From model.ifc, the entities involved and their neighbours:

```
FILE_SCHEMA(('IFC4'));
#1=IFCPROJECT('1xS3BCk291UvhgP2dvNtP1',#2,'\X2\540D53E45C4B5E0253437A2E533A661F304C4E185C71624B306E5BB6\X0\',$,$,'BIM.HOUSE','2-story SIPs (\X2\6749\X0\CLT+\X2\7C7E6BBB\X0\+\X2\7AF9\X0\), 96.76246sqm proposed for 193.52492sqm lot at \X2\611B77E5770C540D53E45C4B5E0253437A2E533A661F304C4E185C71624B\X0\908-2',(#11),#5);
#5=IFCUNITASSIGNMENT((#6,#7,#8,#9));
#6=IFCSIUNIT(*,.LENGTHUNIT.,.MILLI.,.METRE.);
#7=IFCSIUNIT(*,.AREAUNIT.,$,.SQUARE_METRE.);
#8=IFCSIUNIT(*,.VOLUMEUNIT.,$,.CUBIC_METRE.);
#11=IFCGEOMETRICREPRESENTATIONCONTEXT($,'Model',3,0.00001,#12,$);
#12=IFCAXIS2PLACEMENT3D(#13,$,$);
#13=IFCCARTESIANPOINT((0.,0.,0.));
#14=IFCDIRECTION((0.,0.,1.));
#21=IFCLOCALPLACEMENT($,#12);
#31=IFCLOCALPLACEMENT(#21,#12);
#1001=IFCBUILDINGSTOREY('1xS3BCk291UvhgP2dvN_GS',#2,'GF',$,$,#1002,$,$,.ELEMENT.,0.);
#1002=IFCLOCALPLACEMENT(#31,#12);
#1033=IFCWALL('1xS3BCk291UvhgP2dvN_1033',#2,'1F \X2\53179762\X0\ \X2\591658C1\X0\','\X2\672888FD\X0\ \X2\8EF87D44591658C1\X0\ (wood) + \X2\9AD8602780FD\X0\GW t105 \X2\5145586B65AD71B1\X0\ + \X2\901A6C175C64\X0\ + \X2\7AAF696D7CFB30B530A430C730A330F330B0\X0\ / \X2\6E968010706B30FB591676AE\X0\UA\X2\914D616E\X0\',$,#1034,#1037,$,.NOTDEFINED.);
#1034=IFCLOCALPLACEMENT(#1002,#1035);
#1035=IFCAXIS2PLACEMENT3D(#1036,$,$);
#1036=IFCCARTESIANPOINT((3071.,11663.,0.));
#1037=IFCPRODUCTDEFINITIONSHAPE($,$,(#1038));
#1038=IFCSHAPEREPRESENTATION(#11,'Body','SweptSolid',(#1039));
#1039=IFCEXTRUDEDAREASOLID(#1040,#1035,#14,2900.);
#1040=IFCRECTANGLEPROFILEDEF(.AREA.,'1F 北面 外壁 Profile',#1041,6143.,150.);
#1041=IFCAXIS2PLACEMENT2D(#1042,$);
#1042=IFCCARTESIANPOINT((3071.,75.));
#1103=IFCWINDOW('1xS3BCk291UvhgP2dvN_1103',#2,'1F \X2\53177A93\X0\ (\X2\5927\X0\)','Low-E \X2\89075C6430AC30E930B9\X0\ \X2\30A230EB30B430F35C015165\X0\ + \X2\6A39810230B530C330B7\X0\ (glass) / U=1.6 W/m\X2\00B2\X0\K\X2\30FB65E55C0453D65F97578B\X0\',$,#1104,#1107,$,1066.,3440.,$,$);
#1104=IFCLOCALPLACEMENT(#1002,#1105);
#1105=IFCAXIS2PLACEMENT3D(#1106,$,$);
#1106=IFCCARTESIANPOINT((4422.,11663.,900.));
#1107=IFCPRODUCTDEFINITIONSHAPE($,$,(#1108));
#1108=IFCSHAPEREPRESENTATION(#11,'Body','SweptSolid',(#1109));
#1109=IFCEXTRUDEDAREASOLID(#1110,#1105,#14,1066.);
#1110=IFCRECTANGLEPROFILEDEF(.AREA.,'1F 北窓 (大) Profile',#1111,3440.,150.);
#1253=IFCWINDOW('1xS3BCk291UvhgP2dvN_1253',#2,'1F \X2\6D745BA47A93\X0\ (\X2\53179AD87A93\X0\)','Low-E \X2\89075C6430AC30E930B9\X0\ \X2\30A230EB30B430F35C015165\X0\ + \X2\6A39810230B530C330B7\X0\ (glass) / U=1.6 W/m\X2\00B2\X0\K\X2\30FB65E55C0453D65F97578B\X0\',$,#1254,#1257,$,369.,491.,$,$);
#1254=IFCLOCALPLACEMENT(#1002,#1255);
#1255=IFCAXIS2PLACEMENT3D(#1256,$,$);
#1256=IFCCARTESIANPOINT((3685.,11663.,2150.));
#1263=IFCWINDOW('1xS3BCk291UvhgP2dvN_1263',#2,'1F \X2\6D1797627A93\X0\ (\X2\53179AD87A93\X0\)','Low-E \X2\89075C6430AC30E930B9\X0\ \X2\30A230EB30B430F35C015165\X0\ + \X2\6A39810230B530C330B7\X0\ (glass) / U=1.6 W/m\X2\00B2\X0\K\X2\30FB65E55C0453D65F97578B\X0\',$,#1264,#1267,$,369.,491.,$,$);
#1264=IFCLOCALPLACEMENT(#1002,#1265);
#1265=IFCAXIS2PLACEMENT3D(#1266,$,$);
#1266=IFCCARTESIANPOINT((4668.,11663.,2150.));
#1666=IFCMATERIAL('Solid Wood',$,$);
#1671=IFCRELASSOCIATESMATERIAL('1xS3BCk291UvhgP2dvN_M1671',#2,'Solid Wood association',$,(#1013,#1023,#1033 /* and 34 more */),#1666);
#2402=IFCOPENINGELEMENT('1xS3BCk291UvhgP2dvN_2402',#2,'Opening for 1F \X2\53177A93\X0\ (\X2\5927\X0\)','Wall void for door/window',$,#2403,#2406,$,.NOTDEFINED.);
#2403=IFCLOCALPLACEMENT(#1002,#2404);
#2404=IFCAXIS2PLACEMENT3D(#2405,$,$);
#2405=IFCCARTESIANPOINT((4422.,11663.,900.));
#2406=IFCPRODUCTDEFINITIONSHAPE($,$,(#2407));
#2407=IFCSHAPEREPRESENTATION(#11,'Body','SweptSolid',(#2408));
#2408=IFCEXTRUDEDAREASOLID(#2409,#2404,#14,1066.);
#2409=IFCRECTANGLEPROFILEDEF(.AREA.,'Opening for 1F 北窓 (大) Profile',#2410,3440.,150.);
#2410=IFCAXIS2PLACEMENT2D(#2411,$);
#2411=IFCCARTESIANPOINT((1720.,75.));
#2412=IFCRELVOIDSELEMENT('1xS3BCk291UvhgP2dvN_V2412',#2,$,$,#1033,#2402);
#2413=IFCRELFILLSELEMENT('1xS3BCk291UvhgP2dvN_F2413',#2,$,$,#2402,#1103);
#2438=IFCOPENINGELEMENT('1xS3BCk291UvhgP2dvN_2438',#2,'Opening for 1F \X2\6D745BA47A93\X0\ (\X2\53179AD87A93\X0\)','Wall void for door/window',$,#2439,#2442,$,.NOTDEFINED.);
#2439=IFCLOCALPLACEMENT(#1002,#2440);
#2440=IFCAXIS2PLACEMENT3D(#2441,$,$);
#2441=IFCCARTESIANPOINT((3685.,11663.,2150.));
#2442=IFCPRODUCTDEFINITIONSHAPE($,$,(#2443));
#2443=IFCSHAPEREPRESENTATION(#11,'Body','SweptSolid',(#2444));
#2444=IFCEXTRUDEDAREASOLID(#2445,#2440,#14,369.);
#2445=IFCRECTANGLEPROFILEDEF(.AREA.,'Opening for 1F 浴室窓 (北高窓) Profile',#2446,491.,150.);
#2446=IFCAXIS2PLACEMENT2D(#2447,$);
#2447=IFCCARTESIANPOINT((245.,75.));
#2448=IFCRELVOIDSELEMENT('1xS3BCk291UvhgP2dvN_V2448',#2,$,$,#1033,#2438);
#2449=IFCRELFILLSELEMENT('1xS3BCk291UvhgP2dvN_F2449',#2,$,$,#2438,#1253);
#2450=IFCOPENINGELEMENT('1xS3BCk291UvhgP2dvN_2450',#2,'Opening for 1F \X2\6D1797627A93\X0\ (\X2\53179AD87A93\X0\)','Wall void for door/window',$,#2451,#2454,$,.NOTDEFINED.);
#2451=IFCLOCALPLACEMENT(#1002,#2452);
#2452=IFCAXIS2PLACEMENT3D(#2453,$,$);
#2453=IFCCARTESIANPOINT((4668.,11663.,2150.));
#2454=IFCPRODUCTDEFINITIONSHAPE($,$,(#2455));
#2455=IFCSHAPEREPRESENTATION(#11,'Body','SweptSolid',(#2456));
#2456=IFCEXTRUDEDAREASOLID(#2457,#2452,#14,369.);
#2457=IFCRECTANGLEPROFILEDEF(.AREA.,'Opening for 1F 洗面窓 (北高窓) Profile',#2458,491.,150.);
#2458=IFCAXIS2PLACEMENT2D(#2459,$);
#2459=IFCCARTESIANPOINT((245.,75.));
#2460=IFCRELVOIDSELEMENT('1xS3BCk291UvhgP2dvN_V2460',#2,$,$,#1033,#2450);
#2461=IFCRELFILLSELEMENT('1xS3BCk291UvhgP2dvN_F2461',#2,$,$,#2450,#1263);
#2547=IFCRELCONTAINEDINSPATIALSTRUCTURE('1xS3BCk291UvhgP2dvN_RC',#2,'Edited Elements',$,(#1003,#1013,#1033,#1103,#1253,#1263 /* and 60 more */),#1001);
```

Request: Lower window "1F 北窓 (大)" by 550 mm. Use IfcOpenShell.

```python
import numpy as np
import ifcopenshell
import ifcopenshell.api.geometry
import ifcopenshell.util.placement
import ifcopenshell.util.unit

model = ifcopenshell.open("model.ifc")
unit_scale = ifcopenshell.util.unit.calculate_unit_scale(model)

window = model.by_guid("1xS3BCk291UvhgP2dvN_1103")
opening = window.FillsVoids[0].RelatingOpeningElement
dz = -550.0

shift = np.array([0.0, 0.0, dz])
# The window is not placed relative to its opening, so move both.
for product in (opening, window):
    matrix = ifcopenshell.util.placement.get_local_placement(product.ObjectPlacement)
    matrix[:3, 3] += shift
    ifcopenshell.api.geometry.edit_object_placement(model, product=product, matrix=matrix, is_si=False)

print(f"moved by {dz * unit_scale:+.3f} m")

model.write("model_v2.ifc")
```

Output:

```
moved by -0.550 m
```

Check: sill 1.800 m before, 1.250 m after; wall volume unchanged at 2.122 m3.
